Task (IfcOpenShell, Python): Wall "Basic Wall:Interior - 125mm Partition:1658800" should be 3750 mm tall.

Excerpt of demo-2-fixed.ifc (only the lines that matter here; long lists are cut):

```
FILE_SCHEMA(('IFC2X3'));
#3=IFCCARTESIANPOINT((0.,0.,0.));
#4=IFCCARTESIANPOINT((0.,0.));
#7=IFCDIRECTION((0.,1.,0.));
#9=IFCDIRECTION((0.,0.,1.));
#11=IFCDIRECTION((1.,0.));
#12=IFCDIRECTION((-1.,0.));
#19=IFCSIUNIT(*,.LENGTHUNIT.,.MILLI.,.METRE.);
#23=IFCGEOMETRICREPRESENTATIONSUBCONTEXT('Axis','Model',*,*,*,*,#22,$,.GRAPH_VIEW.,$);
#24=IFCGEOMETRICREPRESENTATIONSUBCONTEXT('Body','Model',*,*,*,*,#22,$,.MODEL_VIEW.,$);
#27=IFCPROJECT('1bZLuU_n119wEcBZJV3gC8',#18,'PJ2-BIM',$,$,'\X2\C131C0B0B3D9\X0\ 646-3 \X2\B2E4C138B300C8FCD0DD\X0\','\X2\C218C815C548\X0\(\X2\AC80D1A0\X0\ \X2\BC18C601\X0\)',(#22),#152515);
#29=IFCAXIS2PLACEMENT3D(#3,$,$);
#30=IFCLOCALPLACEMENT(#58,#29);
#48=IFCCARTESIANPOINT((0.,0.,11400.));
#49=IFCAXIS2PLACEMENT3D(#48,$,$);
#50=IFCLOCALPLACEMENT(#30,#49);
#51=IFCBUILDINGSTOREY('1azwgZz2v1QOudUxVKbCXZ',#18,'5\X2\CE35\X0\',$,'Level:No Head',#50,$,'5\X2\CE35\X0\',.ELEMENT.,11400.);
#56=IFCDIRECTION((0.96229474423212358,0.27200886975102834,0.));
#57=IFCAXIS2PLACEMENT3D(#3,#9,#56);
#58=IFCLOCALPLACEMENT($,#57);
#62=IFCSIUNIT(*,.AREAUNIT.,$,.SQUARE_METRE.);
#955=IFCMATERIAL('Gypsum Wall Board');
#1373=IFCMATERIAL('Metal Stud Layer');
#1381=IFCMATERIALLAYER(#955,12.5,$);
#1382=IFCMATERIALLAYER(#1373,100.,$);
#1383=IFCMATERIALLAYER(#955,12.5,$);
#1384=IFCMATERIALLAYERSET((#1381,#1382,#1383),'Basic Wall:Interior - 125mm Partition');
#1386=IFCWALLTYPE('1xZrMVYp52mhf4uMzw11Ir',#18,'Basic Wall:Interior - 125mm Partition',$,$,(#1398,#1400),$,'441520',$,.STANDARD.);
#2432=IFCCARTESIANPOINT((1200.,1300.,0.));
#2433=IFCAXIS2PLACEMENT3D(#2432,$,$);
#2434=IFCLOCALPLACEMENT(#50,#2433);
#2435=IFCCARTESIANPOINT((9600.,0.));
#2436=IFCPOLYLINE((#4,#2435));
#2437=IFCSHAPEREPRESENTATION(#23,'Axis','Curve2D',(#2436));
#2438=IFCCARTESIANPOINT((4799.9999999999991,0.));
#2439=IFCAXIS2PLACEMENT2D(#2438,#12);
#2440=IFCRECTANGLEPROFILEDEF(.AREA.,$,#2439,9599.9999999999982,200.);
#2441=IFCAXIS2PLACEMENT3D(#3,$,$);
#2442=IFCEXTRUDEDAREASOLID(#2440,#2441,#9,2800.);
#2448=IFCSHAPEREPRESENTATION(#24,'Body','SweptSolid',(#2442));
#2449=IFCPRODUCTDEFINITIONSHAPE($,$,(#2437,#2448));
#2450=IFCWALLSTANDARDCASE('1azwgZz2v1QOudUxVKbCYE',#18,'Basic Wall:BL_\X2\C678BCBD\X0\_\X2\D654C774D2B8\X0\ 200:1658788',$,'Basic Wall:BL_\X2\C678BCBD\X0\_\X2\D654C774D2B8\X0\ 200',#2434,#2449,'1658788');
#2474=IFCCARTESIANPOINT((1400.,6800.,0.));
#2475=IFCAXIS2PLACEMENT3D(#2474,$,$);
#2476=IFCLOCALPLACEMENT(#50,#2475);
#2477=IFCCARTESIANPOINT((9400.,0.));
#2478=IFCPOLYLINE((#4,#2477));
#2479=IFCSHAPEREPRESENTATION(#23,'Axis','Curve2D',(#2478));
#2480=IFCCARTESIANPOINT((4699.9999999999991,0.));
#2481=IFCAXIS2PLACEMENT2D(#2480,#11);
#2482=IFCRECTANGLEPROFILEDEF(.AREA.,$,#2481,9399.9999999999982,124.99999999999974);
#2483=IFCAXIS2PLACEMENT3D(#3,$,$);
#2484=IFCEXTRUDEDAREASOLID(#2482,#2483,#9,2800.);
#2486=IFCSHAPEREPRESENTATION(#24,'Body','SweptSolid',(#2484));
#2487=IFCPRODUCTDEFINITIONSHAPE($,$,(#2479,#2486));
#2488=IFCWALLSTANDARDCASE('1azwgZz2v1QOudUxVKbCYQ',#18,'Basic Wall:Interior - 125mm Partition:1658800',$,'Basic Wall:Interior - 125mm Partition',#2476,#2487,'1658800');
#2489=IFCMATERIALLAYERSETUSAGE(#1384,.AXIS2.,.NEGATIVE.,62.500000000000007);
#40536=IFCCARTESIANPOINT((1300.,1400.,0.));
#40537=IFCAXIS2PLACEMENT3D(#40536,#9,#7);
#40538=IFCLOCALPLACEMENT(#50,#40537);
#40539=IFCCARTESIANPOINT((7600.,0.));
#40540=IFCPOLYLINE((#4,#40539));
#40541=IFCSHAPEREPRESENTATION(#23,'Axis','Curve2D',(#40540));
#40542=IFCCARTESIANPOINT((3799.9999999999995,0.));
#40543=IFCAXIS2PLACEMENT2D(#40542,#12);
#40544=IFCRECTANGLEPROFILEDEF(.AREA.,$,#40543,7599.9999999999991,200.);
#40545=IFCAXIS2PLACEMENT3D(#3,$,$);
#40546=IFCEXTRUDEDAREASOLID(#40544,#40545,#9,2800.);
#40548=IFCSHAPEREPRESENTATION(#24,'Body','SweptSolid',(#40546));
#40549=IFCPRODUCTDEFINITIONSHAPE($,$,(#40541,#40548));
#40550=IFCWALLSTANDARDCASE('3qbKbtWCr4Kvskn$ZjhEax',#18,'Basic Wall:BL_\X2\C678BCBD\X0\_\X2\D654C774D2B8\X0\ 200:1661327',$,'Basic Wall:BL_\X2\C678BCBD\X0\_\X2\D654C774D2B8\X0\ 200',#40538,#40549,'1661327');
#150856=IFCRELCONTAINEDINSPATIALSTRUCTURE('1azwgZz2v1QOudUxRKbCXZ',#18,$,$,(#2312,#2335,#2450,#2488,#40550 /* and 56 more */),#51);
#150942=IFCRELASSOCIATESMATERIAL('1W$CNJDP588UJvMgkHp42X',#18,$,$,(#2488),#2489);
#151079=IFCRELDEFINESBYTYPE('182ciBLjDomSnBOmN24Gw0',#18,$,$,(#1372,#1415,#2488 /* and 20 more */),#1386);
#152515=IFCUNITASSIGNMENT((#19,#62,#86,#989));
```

```python
import ifcopenshell
import ifcopenshell.geom
import ifcopenshell.util.representation
import ifcopenshell.util.shape
import ifcopenshell.util.unit

model = ifcopenshell.open("demo-2-fixed.ifc")
unit_scale = ifcopenshell.util.unit.calculate_unit_scale(model)
settings = ifcopenshell.geom.settings()


def volume(element):
    """Net volume in cubic metres, openings subtracted."""
    shape = ifcopenshell.geom.create_shape(settings, element)
    return ifcopenshell.util.shape.get_volume(shape.geometry)


wall = model.by_guid("1azwgZz2v1QOudUxVKbCYQ")
before = volume(wall)

body = ifcopenshell.util.representation.get_representation(wall, "Model", "Body")
solid = body.Items[0]
old_height = solid.Depth
solid.Depth = 3.75 / unit_scale
after = volume(wall)

print(f"height {old_height:g} -> {solid.Depth:g}, volume {before:.3f} -> {after:.3f} m3")

model.write("demo-2-fixed_edited.ifc")
```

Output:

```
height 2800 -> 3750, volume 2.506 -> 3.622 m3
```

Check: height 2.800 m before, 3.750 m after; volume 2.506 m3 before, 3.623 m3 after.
